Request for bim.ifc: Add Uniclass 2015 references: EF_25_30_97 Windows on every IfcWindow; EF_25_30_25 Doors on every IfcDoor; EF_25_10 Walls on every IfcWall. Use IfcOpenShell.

First a look at what the model holds.

```python
import ifcopenshell

model = ifcopenshell.open("bim.ifc")
print(model.schema)
print("classifications:", [c.Name for c in model.by_type("IfcClassification")])
for ifc_class in ("IfcDoor", "IfcRoof", "IfcStair", "IfcWall", "IfcWindow"):
    print(ifc_class, len(model.by_type(ifc_class)))
```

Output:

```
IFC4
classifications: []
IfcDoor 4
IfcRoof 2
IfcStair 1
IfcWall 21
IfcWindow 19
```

```python
import ifcopenshell
import ifcopenshell.api.classification

model = ifcopenshell.open("bim.ifc")

system = ifcopenshell.api.classification.add_classification(model, classification="Uniclass 2015")

codes = {
    "IfcWindow": ("EF_25_30_97", "Windows"),
    "IfcDoor": ("EF_25_30_25", "Doors"),
    "IfcWall": ("EF_25_10", "Walls"),
}
for ifc_class, (code, name) in codes.items():
    products = model.by_type(ifc_class)
    ifcopenshell.api.classification.add_reference(
        model, products=products, classification=system, identification=code, name=name
    )
    print(code, len(products))

model.write("bim-out.ifc")
```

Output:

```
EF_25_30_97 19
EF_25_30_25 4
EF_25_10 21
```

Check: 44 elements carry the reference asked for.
